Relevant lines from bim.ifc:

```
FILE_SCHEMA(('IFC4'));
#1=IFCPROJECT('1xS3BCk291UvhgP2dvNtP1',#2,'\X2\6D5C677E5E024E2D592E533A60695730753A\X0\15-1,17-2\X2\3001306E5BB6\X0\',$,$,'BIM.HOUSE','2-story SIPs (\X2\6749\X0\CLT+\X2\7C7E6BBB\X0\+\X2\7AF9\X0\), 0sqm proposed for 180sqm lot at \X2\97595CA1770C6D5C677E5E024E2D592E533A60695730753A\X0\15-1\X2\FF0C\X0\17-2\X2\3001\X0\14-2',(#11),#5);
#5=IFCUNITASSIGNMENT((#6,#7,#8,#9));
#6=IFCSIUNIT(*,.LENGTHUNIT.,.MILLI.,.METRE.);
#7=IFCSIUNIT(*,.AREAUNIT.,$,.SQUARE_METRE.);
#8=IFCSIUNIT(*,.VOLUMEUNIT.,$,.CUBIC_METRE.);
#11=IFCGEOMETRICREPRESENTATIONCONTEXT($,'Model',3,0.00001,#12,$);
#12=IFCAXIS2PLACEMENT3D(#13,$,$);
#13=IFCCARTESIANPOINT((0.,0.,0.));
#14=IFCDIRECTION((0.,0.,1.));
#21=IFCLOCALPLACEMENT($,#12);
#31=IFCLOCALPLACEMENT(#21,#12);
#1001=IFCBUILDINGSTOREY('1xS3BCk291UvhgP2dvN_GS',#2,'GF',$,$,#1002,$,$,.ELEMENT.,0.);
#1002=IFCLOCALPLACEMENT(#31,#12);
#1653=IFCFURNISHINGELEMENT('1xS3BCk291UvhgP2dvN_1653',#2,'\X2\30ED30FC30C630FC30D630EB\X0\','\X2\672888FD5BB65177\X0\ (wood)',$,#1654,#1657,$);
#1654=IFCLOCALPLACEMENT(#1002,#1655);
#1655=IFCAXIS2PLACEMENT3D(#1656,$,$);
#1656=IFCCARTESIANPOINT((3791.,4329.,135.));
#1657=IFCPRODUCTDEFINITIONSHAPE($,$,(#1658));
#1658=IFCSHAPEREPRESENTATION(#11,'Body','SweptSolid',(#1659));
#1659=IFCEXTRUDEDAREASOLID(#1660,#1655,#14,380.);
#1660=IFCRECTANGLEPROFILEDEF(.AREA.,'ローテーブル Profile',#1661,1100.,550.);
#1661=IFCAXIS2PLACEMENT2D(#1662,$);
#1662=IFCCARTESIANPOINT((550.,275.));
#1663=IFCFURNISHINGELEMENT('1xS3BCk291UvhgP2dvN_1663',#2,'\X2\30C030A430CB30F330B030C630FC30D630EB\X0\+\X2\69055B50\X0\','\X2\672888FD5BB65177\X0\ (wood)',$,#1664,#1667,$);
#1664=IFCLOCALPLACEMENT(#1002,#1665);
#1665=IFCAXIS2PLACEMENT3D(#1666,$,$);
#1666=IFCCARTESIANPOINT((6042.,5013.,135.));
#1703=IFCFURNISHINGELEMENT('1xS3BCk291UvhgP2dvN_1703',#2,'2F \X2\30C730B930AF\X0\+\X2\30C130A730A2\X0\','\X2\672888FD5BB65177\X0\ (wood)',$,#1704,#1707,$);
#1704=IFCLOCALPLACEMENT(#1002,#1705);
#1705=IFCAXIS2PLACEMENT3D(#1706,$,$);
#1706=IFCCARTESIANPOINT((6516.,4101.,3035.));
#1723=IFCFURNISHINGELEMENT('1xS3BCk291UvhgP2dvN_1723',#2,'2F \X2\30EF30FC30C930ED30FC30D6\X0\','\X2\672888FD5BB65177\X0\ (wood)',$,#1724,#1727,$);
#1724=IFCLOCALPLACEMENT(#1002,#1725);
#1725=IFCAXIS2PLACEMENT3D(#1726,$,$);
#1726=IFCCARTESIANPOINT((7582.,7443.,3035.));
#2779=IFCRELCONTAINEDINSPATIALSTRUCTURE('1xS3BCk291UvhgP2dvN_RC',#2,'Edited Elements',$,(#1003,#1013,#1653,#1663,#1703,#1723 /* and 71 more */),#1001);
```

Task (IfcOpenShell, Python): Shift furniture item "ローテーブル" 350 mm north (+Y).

```python
import ifcopenshell
import ifcopenshell.api.geometry
import ifcopenshell.util.placement
import ifcopenshell.util.unit

model = ifcopenshell.open("bim.ifc")
unit_scale = ifcopenshell.util.unit.calculate_unit_scale(model)

item = model.by_guid("1xS3BCk291UvhgP2dvN_1653")
matrix = ifcopenshell.util.placement.get_local_placement(item.ObjectPlacement)
matrix[1, 3] += 0.35 / unit_scale
ifcopenshell.api.geometry.edit_object_placement(model, product=item, matrix=matrix, is_si=False)

print(ifcopenshell.util.placement.get_local_placement(item.ObjectPlacement).round(3) + 0.0)

model.write("bim_rev.ifc")
```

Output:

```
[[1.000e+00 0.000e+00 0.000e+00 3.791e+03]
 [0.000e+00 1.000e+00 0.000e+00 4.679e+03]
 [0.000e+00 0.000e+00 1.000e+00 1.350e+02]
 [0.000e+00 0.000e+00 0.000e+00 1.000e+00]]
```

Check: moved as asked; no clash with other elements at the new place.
